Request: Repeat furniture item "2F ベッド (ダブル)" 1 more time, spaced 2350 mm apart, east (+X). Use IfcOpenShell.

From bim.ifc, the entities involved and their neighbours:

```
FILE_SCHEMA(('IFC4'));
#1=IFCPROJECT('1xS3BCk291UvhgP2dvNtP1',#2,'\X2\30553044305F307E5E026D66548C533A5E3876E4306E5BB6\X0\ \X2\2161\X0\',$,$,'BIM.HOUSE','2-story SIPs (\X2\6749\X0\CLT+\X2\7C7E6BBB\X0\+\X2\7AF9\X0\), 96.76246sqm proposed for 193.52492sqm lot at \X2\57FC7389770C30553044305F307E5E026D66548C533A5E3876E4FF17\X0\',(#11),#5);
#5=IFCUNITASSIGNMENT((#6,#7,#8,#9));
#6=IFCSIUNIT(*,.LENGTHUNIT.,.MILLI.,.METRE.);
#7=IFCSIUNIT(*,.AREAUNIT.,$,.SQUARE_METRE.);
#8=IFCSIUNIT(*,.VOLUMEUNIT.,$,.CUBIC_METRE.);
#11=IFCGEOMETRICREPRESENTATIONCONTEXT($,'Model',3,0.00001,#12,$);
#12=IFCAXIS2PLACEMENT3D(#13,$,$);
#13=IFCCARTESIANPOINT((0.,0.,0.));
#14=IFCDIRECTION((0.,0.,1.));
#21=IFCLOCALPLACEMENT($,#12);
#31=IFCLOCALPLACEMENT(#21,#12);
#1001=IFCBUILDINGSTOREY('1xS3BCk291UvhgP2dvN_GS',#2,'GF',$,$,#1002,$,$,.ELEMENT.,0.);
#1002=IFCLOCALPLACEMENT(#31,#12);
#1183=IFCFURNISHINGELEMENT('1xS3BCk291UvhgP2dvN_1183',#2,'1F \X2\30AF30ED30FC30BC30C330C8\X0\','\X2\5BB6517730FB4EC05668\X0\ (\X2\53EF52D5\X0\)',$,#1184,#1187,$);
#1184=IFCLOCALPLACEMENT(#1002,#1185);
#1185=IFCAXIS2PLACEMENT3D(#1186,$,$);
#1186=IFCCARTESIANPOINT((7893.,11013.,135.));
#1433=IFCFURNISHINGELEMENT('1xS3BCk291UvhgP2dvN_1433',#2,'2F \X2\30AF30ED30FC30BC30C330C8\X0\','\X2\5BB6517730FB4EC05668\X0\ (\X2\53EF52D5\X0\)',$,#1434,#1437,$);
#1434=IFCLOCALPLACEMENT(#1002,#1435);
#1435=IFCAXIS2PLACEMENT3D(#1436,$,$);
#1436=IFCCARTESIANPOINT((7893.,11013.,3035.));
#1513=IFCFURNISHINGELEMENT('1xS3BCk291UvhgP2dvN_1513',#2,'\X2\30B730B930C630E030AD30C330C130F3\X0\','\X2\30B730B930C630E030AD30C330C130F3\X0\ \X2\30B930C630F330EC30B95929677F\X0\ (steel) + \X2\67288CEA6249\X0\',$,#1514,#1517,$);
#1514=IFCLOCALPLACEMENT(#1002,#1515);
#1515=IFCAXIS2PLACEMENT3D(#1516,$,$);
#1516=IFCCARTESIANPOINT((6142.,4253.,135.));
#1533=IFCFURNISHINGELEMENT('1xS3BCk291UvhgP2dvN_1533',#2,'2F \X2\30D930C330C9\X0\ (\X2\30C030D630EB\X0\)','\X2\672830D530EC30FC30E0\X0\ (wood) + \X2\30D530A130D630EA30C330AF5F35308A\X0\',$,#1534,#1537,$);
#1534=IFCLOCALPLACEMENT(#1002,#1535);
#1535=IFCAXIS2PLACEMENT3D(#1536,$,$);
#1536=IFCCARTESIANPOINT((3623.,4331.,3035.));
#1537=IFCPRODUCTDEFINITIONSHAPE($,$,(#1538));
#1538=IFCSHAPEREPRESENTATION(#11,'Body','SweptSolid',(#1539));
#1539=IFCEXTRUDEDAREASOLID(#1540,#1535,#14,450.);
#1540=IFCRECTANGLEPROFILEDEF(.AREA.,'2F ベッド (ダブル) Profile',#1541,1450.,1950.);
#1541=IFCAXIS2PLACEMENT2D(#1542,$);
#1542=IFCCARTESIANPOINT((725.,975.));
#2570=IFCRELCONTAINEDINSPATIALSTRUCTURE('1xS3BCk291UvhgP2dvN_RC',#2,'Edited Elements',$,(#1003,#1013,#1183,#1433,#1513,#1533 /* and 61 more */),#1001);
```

```python
import numpy as np
import ifcopenshell
import ifcopenshell.api.geometry
import ifcopenshell.api.root
import ifcopenshell.util.element
import ifcopenshell.util.placement

model = ifcopenshell.open("bim.ifc")


def reuse_history(source, copy):
    """copy_class also copies each property set's owner history, people and application; keep the originals."""
    for rel in copy.IsDefinedBy:
        if rel.is_a("IfcRelDefinesByProperties") and (history := rel.RelatingPropertyDefinition.OwnerHistory):
            rel.RelatingPropertyDefinition.OwnerHistory = source.OwnerHistory
            ifcopenshell.util.element.remove_deep2(model, history)


source = model.by_id(1533)
base = ifcopenshell.util.placement.get_local_placement(source.ObjectPlacement)
step = np.array([1.0, 0.0, 0.0]) * 2350.0

for i in range(1, 2):
    copy = ifcopenshell.api.root.copy_class(model, product=source)
    copy.Representation = ifcopenshell.util.element.copy_deep(
        model, source.Representation, exclude=["IfcGeometricRepresentationContext", "IfcRepresentationMap"]
    )
    reuse_history(source, copy)
    matrix = base.copy()
    matrix[:3, 3] += i * step
    print("added at", matrix[:3, 3].round(3) + 0.0)
    ifcopenshell.api.geometry.edit_object_placement(model, product=copy, matrix=matrix, is_si=False)

model.write("bim_v2.ifc")
```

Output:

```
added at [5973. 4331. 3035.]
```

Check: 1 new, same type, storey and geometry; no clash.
